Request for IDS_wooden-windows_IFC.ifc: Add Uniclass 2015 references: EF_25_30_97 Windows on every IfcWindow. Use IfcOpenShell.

First a look at what the model holds.

```python
import ifcopenshell

model = ifcopenshell.open("IDS_wooden-windows_IFC.ifc")
print(model.schema)
print("classifications:", [c.Name for c in model.by_type("IfcClassification")])
for ifc_class in ("IfcDoor", "IfcRoof", "IfcStair", "IfcWall", "IfcWindow"):
    print(ifc_class, len(model.by_type(ifc_class)))
```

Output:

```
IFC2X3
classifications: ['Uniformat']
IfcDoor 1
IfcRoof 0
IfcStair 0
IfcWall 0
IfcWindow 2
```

```python
import ifcopenshell
import ifcopenshell.api.classification

model = ifcopenshell.open("IDS_wooden-windows_IFC.ifc")

# IFC2X3 requires Source and Edition and has no link from the project to the system.
system = model.create_entity("IfcClassification", Source="NBS", Edition="2015", Name="Uniclass 2015")

codes = {
    "IfcWindow": ("EF_25_30_97", "Windows"),
}
for ifc_class, (code, name) in codes.items():
    products = model.by_type(ifc_class)
    ifcopenshell.api.classification.add_reference(
        model, products=products, classification=system, identification=code, name=name
    )
    print(code, len(products))

model.write("IDS_wooden-windows_IFC-out.ifc")
```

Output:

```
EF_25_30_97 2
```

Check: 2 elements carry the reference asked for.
